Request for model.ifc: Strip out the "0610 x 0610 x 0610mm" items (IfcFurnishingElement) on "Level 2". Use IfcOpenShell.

First a look at what the model holds.

```python
import ifcopenshell
import ifcopenshell.util.element

model = ifcopenshell.open("model.ifc")
print(model.schema)
storey = next(s for s in model.by_type("IfcBuildingStorey") if s.Name == "Level 2")
furniture = [e for e in ifcopenshell.util.element.get_decomposition(storey) if e.is_a("IfcFurnishingElement")]
seen = {}
for e in furniture:
    element_type = ifcopenshell.util.element.get_type(e)
    name = element_type.Name if element_type not in (None, e) else None
    seen[name] = seen.get(name, 0) + 1
for name, count in sorted(seen.items(), key=str):
    print(count, "x", name)
```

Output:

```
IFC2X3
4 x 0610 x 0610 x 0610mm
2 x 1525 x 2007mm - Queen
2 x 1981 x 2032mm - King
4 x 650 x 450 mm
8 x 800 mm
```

```python
import ifcopenshell
import ifcopenshell.api.root
import ifcopenshell.util.element

model = ifcopenshell.open("model.ifc")

storey = next(s for s in model.by_type("IfcBuildingStorey") if s.Name == "Level 2")
furniture = [e for e in ifcopenshell.util.element.get_decomposition(storey) if e.is_a("IfcFurnishingElement")]
targets = [e for e in furniture if (t := ifcopenshell.util.element.get_type(e)) not in (None, e) and t.Name == "0610 x 0610 x 0610mm"]

for e in targets:
    ifcopenshell.api.root.remove_product(model, product=e)
print(len(targets), "removed")

model.write("model-out.ifc")
```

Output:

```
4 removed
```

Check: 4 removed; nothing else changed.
